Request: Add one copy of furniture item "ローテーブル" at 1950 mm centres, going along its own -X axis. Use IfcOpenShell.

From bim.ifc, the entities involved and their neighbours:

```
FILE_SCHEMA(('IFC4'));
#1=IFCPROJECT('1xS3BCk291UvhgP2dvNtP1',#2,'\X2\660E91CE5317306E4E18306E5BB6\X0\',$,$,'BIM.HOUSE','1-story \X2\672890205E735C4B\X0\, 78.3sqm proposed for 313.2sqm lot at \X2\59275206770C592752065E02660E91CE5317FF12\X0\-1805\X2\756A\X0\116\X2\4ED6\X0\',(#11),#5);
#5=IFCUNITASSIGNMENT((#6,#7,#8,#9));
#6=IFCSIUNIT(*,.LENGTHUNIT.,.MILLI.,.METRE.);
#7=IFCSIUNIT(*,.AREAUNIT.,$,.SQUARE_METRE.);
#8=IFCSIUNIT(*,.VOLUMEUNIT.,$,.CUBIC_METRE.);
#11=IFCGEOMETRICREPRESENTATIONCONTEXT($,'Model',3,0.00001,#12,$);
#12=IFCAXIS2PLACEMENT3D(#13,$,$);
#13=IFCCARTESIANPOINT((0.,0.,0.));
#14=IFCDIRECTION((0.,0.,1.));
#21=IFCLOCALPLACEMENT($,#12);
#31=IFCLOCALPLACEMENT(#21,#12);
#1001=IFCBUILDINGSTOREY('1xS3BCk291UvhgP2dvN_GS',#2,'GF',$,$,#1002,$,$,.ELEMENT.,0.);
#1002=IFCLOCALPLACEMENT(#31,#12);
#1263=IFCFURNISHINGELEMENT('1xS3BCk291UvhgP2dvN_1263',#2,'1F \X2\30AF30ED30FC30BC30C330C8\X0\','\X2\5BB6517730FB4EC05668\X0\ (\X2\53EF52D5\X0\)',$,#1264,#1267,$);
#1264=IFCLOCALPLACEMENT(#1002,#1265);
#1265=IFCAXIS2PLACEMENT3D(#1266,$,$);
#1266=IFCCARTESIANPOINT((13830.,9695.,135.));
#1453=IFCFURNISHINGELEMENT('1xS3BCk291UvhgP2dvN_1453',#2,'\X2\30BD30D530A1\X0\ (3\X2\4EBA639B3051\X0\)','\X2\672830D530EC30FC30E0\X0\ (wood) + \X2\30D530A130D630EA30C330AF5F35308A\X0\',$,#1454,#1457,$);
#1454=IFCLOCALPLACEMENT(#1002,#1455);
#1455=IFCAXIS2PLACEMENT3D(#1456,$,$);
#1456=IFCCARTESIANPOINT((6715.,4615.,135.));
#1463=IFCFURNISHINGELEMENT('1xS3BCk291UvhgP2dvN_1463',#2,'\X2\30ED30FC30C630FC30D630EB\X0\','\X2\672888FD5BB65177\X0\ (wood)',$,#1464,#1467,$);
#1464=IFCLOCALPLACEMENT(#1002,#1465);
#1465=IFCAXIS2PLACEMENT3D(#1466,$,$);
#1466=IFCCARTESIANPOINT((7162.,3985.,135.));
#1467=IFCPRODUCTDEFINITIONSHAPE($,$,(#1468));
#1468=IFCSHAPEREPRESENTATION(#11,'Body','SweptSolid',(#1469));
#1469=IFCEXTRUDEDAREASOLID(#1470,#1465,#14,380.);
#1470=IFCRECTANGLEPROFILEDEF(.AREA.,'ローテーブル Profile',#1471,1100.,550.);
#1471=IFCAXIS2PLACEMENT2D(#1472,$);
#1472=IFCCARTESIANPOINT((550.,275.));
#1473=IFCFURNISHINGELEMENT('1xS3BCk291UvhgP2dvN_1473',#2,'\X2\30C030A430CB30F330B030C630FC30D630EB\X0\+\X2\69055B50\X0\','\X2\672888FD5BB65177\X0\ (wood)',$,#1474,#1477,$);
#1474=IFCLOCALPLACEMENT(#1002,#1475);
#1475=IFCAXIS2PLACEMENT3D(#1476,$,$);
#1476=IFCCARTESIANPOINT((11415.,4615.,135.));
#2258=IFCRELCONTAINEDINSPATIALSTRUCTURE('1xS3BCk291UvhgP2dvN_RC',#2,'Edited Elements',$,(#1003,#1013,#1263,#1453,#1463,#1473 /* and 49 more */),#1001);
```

```python
import ifcopenshell
import ifcopenshell.api.geometry
import ifcopenshell.api.root
import ifcopenshell.util.element
import ifcopenshell.util.placement

model = ifcopenshell.open("bim.ifc")


def reuse_history(source, copy):
    """copy_class also copies each property set's owner history, people and application; keep the originals."""
    for rel in copy.IsDefinedBy:
        if rel.is_a("IfcRelDefinesByProperties") and (history := rel.RelatingPropertyDefinition.OwnerHistory):
            rel.RelatingPropertyDefinition.OwnerHistory = source.OwnerHistory
            ifcopenshell.util.element.remove_deep2(model, history)


source = model.by_guid("1xS3BCk291UvhgP2dvN_1463")
base = ifcopenshell.util.placement.get_local_placement(source.ObjectPlacement)
step = -base[:3, 0] * 1950.0

for i in range(1, 2):
    copy = ifcopenshell.api.root.copy_class(model, product=source)
    copy.Representation = ifcopenshell.util.element.copy_deep(
        model, source.Representation, exclude=["IfcGeometricRepresentationContext", "IfcRepresentationMap"]
    )
    reuse_history(source, copy)
    matrix = base.copy()
    matrix[:3, 3] += i * step
    print("added at", matrix[:3, 3].round(3) + 0.0)
    ifcopenshell.api.geometry.edit_object_placement(model, product=copy, matrix=matrix, is_si=False)

model.write("bim_rev.ifc")
```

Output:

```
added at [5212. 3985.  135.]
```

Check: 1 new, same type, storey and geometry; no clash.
